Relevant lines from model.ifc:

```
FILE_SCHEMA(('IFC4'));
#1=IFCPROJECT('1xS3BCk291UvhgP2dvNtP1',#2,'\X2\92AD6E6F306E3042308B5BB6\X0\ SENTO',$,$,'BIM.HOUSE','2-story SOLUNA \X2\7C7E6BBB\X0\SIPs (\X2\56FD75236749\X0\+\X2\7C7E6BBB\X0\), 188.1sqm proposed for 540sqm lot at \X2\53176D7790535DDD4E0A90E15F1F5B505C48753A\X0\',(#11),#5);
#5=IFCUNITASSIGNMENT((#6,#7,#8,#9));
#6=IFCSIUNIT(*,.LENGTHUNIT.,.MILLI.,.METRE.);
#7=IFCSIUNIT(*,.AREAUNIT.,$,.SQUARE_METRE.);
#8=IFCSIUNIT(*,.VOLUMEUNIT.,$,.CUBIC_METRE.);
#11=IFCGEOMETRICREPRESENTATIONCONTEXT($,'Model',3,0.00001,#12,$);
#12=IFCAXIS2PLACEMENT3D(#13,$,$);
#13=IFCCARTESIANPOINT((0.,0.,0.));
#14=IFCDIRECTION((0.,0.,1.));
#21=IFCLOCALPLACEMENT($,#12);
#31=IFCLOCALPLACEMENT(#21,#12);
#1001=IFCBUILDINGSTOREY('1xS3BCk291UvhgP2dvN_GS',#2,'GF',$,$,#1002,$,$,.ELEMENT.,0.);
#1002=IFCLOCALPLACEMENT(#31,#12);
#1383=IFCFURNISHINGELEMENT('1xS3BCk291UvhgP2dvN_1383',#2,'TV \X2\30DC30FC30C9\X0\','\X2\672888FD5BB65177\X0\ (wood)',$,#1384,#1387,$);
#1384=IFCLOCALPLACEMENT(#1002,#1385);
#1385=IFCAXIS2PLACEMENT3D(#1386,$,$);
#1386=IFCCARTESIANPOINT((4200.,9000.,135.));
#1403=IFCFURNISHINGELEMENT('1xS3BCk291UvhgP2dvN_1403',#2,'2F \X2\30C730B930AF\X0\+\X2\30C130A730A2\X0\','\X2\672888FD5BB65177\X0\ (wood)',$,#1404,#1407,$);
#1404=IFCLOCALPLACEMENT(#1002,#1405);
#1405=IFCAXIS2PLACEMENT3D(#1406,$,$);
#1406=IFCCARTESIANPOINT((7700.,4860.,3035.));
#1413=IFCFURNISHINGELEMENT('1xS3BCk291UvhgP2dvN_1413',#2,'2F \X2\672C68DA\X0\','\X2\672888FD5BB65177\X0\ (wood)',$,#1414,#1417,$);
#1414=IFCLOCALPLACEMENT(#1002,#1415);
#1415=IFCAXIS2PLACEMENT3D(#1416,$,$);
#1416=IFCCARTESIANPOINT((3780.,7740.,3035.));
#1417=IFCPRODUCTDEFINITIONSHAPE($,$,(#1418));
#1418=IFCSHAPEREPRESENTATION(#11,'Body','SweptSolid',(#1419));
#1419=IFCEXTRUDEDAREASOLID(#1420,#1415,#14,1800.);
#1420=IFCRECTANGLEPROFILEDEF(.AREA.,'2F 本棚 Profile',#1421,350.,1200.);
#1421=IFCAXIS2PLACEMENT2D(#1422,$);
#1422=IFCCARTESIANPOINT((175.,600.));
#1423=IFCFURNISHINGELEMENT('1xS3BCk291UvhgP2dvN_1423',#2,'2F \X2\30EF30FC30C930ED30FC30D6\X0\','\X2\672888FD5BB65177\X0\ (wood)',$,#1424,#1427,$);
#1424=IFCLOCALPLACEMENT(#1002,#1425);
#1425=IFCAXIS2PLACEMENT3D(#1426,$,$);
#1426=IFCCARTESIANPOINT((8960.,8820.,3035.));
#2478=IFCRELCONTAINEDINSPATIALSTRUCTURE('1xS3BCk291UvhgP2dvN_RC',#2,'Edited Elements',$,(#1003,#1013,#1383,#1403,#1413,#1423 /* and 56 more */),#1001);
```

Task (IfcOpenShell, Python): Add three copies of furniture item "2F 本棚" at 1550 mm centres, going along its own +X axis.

```python
import ifcopenshell
import ifcopenshell.api.geometry
import ifcopenshell.api.root
import ifcopenshell.util.element
import ifcopenshell.util.placement
import ifcopenshell.util.unit

model = ifcopenshell.open("model.ifc")
unit_scale = ifcopenshell.util.unit.calculate_unit_scale(model)


def reuse_history(source, copy):
    """copy_class also copies each property set's owner history, people and application; keep the originals."""
    for rel in copy.IsDefinedBy:
        if rel.is_a("IfcRelDefinesByProperties") and (history := rel.RelatingPropertyDefinition.OwnerHistory):
            rel.RelatingPropertyDefinition.OwnerHistory = source.OwnerHistory
            ifcopenshell.util.element.remove_deep2(model, history)


source = model.by_guid("1xS3BCk291UvhgP2dvN_1413")
base = ifcopenshell.util.placement.get_local_placement(source.ObjectPlacement)
step = base[:3, 0] * 1.55 / unit_scale

for i in range(1, 4):
    copy = ifcopenshell.api.root.copy_class(model, product=source)
    copy.Representation = ifcopenshell.util.element.copy_deep(
        model, source.Representation, exclude=["IfcGeometricRepresentationContext", "IfcRepresentationMap"]
    )
    reuse_history(source, copy)
    matrix = base.copy()
    matrix[:3, 3] += i * step
    print("added at", matrix[:3, 3].round(3) + 0.0)
    ifcopenshell.api.geometry.edit_object_placement(model, product=copy, matrix=matrix, is_si=False)

model.write("model_rev.ifc")
```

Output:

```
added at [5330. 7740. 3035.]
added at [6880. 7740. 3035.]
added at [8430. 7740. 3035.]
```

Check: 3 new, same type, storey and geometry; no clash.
